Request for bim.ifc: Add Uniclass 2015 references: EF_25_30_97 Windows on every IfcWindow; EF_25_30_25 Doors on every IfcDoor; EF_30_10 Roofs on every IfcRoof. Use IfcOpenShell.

First a look at what the model holds.

```python
import ifcopenshell

model = ifcopenshell.open("bim.ifc")
print(model.schema)
print("classifications:", [c.Name for c in model.by_type("IfcClassification")])
for ifc_class in ("IfcDoor", "IfcRoof", "IfcStair", "IfcWall", "IfcWindow"):
    print(ifc_class, len(model.by_type(ifc_class)))
```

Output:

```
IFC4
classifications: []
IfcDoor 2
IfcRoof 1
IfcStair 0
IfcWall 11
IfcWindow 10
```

```python
import ifcopenshell
import ifcopenshell.api.classification

model = ifcopenshell.open("bim.ifc")

system = ifcopenshell.api.classification.add_classification(model, classification="Uniclass 2015")

codes = {
    "IfcWindow": ("EF_25_30_97", "Windows"),
    "IfcDoor": ("EF_25_30_25", "Doors"),
    "IfcRoof": ("EF_30_10", "Roofs"),
}
for ifc_class, (code, name) in codes.items():
    products = model.by_type(ifc_class)
    ifcopenshell.api.classification.add_reference(
        model, products=products, classification=system, identification=code, name=name
    )
    print(code, len(products))

model.write("bim_edited.ifc")
```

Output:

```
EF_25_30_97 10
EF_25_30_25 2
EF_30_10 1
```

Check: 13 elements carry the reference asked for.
